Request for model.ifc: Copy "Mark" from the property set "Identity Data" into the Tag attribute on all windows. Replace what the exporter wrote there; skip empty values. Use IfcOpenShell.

First a look at what the model holds.

```python
import ifcopenshell
import ifcopenshell.util.element

model = ifcopenshell.open("model.ifc")
print(model.schema)
windows = model.by_type("IfcWindow")
print(len(windows), "windows")
for e in windows[:8]:
    source = ifcopenshell.util.element.get_pset(e, "Identity Data", "Mark")
    target = e.Tag
    print(e.id(), repr(source), repr(target), sep=" | ")
```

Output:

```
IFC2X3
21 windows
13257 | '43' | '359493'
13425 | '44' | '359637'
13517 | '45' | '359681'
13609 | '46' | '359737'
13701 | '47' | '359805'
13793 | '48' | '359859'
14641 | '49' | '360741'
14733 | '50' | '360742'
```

```python
import ifcopenshell
import ifcopenshell.util.element

model = ifcopenshell.open("model.ifc")

count = 0
for e in model.by_type("IfcWindow"):
    value = ifcopenshell.util.element.get_pset(e, "Identity Data", "Mark")
    current = e.Tag
    if not value or not value.strip() or current == value:
        continue
    e.Tag = value
    count += 1

print(count, "windows updated")

model.write("model_edited.ifc")
```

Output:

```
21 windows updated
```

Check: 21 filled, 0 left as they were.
